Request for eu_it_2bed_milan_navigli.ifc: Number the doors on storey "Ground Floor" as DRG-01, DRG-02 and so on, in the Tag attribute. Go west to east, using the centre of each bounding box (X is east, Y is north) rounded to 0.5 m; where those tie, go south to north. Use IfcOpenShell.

First a look at what the model holds.

```python
import ifcopenshell
import ifcopenshell.util.element
import ifcopenshell.util.placement

model = ifcopenshell.open("eu_it_2bed_milan_navigli.ifc")
print(model.schema)
storey = next(s for s in model.by_type("IfcBuildingStorey") if s.Name == "Ground Floor")
doors = [e for e in ifcopenshell.util.element.get_decomposition(storey) if e.is_a("IfcDoor")]
for e in sorted(doors, key=lambda e: e.id()):
    origin = ifcopenshell.util.placement.get_local_placement(e.ObjectPlacement)[:3, 3]
    print(e.id(), e.Tag, e.Name, origin.round(2) + 0.0, sep=" | ")
```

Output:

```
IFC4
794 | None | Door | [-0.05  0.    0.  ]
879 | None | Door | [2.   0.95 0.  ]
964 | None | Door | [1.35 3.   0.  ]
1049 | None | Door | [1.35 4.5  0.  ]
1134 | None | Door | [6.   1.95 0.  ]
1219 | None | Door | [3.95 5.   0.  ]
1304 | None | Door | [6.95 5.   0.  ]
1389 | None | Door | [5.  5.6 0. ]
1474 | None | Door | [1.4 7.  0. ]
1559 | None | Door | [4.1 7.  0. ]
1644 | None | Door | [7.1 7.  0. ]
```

```python
import ifcopenshell
import ifcopenshell.geom
import ifcopenshell.util.element
import ifcopenshell.util.shape

model = ifcopenshell.open("eu_it_2bed_milan_navigli.ifc")
settings = ifcopenshell.geom.settings()
settings.set("use-world-coords", True)


def centre(element):
    shape = ifcopenshell.geom.create_shape(settings, element)
    return ifcopenshell.util.shape.get_bbox_centroid(shape.geometry)


storey = next(s for s in model.by_type("IfcBuildingStorey") if s.Name == "Ground Floor")
doors = [e for e in ifcopenshell.util.element.get_decomposition(storey) if e.is_a("IfcDoor")]

# Insertion points can sit at a corner or the storey origin, so sort by the geometry (in metres).
centres = {e: centre(e) for e in doors}
doors.sort(key=lambda e: (round(centres[e][0] / 0.5), centres[e][1]))

for i, e in enumerate(doors, start=1):
    number = f"DRG-{i:02d}"
    e.Tag = number
    print(e.id(), number)

model.write("eu_it_2bed_milan_navigli-out.ifc")
```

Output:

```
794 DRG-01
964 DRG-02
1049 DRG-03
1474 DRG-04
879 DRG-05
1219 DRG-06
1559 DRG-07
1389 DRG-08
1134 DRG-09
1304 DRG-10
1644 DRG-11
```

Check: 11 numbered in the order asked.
